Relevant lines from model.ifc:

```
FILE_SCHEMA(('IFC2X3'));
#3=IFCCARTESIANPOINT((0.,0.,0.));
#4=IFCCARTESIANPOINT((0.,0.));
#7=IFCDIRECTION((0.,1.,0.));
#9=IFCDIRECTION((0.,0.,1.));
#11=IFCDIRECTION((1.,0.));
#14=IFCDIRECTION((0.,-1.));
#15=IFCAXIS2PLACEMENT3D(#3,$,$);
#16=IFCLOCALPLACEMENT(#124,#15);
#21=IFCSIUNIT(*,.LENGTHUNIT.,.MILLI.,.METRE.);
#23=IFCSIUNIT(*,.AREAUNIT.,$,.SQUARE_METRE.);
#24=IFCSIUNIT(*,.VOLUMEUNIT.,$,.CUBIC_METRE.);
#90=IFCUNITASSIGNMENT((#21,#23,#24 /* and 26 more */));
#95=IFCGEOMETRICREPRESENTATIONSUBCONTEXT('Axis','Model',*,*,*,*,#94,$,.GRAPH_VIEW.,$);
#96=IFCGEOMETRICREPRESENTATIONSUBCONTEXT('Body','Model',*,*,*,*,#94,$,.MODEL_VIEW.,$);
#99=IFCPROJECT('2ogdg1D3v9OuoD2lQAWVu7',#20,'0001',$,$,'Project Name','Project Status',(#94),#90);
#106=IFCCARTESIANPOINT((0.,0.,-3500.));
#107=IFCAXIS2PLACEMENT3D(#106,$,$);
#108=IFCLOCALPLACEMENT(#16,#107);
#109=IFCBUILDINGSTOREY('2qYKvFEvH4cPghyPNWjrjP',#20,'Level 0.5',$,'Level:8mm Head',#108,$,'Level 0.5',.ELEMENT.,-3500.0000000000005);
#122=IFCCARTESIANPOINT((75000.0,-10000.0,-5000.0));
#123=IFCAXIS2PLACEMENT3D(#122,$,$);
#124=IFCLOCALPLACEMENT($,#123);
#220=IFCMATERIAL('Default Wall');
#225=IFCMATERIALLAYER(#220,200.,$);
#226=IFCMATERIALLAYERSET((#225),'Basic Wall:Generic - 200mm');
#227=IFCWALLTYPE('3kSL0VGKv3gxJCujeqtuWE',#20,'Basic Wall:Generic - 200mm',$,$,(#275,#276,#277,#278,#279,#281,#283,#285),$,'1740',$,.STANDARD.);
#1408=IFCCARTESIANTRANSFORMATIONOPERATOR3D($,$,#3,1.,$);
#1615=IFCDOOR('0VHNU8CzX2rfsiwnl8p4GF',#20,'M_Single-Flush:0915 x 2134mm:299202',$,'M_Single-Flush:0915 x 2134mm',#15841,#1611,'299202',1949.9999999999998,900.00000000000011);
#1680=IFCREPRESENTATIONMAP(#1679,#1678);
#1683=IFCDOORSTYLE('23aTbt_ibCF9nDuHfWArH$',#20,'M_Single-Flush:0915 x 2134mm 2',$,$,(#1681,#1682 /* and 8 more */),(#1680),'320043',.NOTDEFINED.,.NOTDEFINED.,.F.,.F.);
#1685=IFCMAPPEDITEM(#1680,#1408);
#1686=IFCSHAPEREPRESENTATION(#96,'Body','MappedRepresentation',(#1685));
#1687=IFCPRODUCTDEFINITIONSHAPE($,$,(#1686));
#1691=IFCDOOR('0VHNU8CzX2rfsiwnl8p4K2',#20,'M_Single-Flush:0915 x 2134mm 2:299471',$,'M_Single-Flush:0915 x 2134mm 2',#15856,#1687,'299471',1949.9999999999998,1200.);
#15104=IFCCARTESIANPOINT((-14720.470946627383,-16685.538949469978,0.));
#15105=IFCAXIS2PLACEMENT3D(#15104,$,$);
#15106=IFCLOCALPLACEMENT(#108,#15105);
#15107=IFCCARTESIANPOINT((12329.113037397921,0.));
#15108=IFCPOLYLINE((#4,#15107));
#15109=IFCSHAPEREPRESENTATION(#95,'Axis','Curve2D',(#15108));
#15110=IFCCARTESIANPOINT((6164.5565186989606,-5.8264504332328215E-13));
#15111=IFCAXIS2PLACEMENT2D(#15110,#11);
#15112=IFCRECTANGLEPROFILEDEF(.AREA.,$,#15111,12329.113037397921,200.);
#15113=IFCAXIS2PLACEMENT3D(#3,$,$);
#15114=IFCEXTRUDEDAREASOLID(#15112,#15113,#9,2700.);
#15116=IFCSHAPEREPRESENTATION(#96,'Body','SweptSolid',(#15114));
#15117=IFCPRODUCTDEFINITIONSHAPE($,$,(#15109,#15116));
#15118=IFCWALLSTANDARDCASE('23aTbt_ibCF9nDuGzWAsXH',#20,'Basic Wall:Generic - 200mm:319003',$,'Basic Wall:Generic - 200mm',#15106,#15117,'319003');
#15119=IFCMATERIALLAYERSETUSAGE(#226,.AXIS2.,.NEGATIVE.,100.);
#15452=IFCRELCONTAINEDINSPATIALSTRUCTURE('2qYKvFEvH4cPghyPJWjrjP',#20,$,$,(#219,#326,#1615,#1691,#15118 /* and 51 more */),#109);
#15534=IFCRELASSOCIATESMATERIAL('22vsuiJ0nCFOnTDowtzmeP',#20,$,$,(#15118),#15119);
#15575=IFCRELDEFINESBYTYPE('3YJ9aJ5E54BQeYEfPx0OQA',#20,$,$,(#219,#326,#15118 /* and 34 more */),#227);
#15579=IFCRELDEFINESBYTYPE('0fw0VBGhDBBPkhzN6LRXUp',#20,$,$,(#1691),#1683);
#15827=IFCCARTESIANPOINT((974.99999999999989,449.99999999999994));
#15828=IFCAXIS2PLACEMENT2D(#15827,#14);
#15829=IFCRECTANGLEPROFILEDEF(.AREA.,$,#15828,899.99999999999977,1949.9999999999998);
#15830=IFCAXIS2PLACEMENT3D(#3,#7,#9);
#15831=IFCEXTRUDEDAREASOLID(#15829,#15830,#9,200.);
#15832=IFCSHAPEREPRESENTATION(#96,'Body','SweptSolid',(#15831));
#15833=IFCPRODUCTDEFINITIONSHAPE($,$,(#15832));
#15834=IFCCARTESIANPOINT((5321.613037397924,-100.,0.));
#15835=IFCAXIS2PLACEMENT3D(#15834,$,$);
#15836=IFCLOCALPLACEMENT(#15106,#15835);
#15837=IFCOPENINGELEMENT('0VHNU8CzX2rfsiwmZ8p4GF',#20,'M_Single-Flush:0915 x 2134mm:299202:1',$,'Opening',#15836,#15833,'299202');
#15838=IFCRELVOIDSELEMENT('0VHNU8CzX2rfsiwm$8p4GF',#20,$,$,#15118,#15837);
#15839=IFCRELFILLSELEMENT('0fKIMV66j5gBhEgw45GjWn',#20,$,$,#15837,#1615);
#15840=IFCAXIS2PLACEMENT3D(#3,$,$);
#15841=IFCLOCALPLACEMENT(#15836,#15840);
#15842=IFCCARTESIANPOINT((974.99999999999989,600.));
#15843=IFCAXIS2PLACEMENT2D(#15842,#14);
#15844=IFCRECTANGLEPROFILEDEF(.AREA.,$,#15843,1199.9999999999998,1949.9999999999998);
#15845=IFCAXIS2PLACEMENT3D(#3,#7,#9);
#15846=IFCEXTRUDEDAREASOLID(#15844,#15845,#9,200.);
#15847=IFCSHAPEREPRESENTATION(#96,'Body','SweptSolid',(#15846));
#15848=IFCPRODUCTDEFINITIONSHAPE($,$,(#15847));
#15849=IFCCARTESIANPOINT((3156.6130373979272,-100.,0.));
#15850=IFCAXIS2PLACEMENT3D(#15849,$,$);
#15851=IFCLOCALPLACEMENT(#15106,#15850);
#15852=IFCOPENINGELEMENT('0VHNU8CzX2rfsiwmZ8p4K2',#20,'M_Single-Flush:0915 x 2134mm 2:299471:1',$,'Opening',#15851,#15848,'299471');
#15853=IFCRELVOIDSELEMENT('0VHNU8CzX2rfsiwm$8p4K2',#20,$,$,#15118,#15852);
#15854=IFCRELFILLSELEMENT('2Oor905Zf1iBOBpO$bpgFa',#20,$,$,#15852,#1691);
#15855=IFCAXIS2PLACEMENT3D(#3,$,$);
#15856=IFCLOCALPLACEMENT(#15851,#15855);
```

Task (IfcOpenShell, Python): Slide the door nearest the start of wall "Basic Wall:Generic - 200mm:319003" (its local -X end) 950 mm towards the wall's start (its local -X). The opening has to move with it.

```python
import ifcopenshell
import ifcopenshell.api.geometry
import ifcopenshell.util.placement
import ifcopenshell.util.unit

model = ifcopenshell.open("model.ifc")
unit_scale = ifcopenshell.util.unit.calculate_unit_scale(model)

door = model.by_guid("0VHNU8CzX2rfsiwnl8p4K2")
opening = door.FillsVoids[0].RelatingOpeningElement
wall = opening.VoidsElements[0].RelatingBuildingElement

wall_matrix = ifcopenshell.util.placement.get_local_placement(wall.ObjectPlacement)
shift = wall_matrix[:3, 0] * -0.95 / unit_scale
before = ifcopenshell.util.placement.get_local_placement(door.ObjectPlacement)[:3, 3].copy()

# The door is placed relative to its opening, so it follows when the opening moves.
matrix = ifcopenshell.util.placement.get_local_placement(opening.ObjectPlacement)
matrix[:3, 3] += shift
ifcopenshell.api.geometry.edit_object_placement(
    model, product=opening, matrix=matrix, is_si=False, should_transform_children=True
)

after = ifcopenshell.util.placement.get_local_placement(door.ObjectPlacement)[:3, 3]
print("door moved by", (after - before).round(3) + 0.0)

model.write("model_edited.ifc")
```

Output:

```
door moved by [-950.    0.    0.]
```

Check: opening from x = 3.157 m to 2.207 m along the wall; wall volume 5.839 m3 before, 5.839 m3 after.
